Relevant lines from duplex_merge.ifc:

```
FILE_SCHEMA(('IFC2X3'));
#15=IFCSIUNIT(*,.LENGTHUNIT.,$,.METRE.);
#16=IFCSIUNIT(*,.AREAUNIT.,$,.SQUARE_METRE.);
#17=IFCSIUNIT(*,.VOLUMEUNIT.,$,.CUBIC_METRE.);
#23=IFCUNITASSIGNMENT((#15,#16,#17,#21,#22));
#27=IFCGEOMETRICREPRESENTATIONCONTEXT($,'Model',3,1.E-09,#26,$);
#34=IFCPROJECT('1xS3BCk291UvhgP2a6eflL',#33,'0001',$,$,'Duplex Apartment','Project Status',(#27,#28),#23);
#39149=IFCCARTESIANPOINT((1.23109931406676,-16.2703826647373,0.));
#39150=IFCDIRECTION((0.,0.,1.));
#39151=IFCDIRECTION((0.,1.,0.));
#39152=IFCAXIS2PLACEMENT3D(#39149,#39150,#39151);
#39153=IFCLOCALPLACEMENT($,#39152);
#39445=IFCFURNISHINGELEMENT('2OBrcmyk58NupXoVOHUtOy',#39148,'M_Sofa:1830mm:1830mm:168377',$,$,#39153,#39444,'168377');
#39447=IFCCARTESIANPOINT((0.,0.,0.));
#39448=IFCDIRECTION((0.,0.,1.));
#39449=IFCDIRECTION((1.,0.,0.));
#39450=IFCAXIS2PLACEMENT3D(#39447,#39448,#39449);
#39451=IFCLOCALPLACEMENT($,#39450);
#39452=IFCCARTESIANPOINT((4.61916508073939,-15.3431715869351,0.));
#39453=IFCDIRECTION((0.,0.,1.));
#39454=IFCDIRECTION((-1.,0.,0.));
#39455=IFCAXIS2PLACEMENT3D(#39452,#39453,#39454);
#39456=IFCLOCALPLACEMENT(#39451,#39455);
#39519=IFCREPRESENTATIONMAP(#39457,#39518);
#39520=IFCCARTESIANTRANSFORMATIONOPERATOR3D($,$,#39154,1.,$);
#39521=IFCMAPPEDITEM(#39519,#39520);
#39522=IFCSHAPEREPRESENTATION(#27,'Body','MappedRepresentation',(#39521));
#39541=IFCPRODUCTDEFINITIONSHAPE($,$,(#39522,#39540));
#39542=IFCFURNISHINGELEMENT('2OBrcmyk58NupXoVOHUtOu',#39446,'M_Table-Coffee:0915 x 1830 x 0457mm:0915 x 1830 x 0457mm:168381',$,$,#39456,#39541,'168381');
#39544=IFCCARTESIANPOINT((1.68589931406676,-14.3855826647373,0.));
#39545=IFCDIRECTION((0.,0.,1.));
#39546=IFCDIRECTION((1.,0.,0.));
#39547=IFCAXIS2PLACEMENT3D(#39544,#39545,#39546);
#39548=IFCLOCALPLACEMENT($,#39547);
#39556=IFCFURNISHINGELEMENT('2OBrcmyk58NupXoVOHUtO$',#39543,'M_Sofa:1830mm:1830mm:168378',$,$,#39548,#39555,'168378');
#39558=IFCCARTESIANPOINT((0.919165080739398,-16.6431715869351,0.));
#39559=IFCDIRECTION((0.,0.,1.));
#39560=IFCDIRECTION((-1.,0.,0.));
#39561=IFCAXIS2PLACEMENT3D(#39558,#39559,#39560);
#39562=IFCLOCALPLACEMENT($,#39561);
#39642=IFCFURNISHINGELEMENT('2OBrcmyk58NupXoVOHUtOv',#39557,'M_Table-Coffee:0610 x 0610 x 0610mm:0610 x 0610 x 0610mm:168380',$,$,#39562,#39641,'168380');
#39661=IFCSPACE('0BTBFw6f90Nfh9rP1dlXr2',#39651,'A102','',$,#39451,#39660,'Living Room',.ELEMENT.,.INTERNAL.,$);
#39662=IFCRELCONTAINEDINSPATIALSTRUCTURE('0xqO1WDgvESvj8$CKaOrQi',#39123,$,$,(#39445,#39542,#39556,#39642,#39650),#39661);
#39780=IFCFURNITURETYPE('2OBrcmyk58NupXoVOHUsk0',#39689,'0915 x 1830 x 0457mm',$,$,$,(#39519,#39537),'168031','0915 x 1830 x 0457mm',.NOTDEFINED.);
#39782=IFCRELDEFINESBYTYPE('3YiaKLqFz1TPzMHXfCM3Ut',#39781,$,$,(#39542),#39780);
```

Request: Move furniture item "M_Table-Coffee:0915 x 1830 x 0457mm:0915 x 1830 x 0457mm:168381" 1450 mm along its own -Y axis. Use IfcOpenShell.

```python
import ifcopenshell
import ifcopenshell.api.geometry
import ifcopenshell.util.placement
import ifcopenshell.util.unit

model = ifcopenshell.open("duplex_merge.ifc")
unit_scale = ifcopenshell.util.unit.calculate_unit_scale(model)

item = model.by_guid("2OBrcmyk58NupXoVOHUtOu")
matrix = ifcopenshell.util.placement.get_local_placement(item.ObjectPlacement)
matrix[:3, 3] -= matrix[:3, 1] * 1.45 / unit_scale
ifcopenshell.api.geometry.edit_object_placement(model, product=item, matrix=matrix, is_si=False)

print(ifcopenshell.util.placement.get_local_placement(item.ObjectPlacement).round(3) + 0.0)

model.write("duplex_merge_v2.ifc")
```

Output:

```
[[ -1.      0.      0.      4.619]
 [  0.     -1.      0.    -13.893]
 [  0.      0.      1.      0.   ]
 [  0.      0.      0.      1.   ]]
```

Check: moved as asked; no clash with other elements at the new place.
